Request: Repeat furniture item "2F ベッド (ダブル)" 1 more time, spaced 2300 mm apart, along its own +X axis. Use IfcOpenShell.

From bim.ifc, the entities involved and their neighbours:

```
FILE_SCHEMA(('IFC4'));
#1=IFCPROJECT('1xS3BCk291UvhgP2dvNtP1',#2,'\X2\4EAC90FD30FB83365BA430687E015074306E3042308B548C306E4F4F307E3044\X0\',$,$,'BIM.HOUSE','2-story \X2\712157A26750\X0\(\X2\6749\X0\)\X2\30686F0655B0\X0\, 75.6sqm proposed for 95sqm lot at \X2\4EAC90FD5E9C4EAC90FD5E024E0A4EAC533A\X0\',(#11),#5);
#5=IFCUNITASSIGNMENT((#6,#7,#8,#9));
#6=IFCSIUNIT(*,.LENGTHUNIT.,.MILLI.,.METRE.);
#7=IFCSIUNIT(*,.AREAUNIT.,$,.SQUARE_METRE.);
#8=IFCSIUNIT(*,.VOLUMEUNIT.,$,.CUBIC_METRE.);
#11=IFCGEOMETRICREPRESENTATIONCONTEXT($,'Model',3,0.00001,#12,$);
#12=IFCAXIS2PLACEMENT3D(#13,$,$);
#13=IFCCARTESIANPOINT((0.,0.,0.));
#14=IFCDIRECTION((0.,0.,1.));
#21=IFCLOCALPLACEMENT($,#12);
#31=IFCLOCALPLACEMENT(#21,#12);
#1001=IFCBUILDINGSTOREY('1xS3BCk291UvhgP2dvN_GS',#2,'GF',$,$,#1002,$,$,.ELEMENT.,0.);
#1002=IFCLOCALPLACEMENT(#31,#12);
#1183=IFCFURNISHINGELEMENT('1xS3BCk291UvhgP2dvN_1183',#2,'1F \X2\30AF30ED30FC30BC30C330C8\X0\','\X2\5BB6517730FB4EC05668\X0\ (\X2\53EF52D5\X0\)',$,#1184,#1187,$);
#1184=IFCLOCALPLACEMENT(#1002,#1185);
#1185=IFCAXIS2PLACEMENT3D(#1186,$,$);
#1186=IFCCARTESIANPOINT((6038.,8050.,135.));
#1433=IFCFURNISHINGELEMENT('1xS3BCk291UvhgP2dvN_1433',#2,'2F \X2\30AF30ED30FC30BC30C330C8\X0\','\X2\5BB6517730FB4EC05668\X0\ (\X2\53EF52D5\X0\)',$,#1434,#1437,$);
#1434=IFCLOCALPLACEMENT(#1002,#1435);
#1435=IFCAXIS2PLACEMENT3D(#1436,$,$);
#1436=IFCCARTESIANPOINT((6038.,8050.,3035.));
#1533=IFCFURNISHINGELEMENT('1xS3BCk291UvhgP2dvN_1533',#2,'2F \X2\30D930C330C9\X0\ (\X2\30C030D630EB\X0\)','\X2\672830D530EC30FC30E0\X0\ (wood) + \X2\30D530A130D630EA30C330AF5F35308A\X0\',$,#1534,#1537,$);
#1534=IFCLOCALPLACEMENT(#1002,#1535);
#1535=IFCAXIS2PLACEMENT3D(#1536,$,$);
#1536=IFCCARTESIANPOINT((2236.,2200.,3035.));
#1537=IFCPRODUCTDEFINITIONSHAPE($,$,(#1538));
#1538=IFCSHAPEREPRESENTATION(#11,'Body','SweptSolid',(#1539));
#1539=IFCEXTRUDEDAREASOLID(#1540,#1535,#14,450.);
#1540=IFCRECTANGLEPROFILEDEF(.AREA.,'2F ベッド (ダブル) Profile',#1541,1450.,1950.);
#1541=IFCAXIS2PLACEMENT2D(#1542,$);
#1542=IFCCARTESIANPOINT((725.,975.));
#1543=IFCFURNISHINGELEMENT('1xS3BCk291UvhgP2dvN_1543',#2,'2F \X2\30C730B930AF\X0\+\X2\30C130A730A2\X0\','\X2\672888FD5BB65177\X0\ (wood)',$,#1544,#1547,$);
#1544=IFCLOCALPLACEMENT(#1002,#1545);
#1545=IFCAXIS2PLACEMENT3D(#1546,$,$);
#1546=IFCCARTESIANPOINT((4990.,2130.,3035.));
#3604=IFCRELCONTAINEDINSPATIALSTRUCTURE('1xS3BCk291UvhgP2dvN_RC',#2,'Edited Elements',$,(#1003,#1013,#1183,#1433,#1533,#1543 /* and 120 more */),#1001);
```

```python
import ifcopenshell
import ifcopenshell.api.geometry
import ifcopenshell.api.root
import ifcopenshell.util.element
import ifcopenshell.util.placement
import ifcopenshell.util.unit

model = ifcopenshell.open("bim.ifc")
unit_scale = ifcopenshell.util.unit.calculate_unit_scale(model)


def reuse_history(source, copy):
    """copy_class also copies each property set's owner history, people and application; keep the originals."""
    for rel in copy.IsDefinedBy:
        if rel.is_a("IfcRelDefinesByProperties") and (history := rel.RelatingPropertyDefinition.OwnerHistory):
            rel.RelatingPropertyDefinition.OwnerHistory = source.OwnerHistory
            ifcopenshell.util.element.remove_deep2(model, history)


source = model.by_guid("1xS3BCk291UvhgP2dvN_1533")
base = ifcopenshell.util.placement.get_local_placement(source.ObjectPlacement)
step = base[:3, 0] * 2.3 / unit_scale

for i in range(1, 2):
    copy = ifcopenshell.api.root.copy_class(model, product=source)
    copy.Representation = ifcopenshell.util.element.copy_deep(
        model, source.Representation, exclude=["IfcGeometricRepresentationContext", "IfcRepresentationMap"]
    )
    reuse_history(source, copy)
    matrix = base.copy()
    matrix[:3, 3] += i * step
    print("added at", matrix[:3, 3].round(3) + 0.0)
    ifcopenshell.api.geometry.edit_object_placement(model, product=copy, matrix=matrix, is_si=False)

model.write("bim_rev.ifc")
```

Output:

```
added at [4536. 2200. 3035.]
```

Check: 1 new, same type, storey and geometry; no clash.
